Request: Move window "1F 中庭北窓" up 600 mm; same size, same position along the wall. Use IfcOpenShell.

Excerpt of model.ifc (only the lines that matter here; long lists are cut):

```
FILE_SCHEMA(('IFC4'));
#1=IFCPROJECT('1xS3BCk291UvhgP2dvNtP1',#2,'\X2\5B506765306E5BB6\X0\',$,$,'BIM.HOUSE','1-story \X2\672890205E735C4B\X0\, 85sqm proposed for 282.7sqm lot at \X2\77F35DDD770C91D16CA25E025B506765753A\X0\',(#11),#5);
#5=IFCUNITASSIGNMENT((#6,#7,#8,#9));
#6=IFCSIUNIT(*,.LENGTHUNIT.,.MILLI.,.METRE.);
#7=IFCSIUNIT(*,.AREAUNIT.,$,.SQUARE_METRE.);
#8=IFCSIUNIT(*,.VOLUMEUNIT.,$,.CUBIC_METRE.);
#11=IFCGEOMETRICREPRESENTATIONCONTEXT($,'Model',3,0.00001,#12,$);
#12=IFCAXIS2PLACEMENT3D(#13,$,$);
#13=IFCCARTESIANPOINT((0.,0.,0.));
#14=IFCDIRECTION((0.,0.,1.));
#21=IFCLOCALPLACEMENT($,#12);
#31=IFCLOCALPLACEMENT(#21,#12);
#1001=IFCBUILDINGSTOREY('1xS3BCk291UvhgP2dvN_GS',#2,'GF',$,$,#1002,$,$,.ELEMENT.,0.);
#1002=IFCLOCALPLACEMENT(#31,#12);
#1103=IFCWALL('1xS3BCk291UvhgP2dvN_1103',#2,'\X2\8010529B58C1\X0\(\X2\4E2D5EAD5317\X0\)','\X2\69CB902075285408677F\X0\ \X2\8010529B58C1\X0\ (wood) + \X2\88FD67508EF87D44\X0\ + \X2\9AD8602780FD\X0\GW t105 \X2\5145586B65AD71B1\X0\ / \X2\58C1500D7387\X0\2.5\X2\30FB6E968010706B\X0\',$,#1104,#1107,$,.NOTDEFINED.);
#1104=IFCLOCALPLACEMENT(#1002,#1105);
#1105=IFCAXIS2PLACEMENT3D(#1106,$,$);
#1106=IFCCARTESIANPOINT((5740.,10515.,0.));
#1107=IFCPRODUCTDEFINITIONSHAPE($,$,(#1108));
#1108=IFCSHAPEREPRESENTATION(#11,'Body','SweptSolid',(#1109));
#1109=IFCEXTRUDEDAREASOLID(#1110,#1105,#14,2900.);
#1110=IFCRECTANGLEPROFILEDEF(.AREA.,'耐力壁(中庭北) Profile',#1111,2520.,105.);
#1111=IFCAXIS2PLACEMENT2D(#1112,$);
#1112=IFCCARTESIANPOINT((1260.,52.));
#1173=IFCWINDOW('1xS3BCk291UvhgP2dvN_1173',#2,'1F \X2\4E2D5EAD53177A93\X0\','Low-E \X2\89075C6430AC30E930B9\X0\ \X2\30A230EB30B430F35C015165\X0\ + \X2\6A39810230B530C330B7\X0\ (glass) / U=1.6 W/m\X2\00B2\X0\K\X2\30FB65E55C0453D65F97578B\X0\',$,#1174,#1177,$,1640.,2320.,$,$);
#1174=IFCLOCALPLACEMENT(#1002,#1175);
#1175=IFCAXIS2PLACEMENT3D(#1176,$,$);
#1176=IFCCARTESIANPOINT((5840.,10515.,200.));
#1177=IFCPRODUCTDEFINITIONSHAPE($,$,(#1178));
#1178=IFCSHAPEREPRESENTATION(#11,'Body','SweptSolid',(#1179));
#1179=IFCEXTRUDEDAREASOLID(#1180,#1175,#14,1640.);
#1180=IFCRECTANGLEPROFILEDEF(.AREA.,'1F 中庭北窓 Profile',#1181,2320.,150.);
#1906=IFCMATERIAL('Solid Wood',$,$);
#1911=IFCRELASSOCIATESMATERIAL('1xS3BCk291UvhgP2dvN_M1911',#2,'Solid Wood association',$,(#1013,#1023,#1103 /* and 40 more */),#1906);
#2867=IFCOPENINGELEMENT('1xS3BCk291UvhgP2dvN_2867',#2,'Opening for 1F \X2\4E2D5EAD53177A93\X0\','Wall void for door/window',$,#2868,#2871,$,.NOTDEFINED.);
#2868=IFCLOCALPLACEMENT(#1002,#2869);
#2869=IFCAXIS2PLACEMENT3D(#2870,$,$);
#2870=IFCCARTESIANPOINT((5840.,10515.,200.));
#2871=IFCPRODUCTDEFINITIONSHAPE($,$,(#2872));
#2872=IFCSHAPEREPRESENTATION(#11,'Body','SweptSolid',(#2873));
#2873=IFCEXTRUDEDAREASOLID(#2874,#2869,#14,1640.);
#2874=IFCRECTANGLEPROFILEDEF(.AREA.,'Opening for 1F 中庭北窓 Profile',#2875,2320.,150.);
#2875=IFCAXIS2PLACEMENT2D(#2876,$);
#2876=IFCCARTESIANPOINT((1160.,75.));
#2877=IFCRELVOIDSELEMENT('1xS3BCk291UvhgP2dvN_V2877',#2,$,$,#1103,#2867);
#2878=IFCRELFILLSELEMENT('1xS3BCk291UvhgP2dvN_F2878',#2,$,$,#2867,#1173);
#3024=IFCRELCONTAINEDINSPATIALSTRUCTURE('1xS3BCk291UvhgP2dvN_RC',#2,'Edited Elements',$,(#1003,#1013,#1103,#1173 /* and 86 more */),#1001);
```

```python
import numpy as np
import ifcopenshell
import ifcopenshell.api.geometry
import ifcopenshell.util.placement
import ifcopenshell.util.unit

model = ifcopenshell.open("model.ifc")
unit_scale = ifcopenshell.util.unit.calculate_unit_scale(model)

window = model.by_guid("1xS3BCk291UvhgP2dvN_1173")
opening = window.FillsVoids[0].RelatingOpeningElement
dz = 600.0

shift = np.array([0.0, 0.0, dz])
# The window is not placed relative to its opening, so move both.
for product in (opening, window):
    matrix = ifcopenshell.util.placement.get_local_placement(product.ObjectPlacement)
    matrix[:3, 3] += shift
    ifcopenshell.api.geometry.edit_object_placement(model, product=product, matrix=matrix, is_si=False)

print(f"moved by {dz * unit_scale:+.3f} m")

model.write("model_updated.ifc")
```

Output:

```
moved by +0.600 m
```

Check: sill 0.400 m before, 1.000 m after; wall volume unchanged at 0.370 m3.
